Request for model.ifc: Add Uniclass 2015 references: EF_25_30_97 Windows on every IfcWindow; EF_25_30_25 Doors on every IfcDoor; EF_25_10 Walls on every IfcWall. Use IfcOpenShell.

First a look at what the model holds.

```python
import ifcopenshell

model = ifcopenshell.open("model.ifc")
print(model.schema)
print("classifications:", [c.Name for c in model.by_type("IfcClassification")])
for ifc_class in ("IfcDoor", "IfcRoof", "IfcStair", "IfcWall", "IfcWindow"):
    print(ifc_class, len(model.by_type(ifc_class)))
```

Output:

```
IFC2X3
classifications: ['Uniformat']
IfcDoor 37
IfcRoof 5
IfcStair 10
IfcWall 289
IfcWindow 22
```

```python
import ifcopenshell
import ifcopenshell.api.classification

model = ifcopenshell.open("model.ifc")

# IFC2X3 requires Source and Edition and has no link from the project to the system.
system = model.create_entity("IfcClassification", Source="NBS", Edition="2015", Name="Uniclass 2015")

codes = {
    "IfcWindow": ("EF_25_30_97", "Windows"),
    "IfcDoor": ("EF_25_30_25", "Doors"),
    "IfcWall": ("EF_25_10", "Walls"),
}
for ifc_class, (code, name) in codes.items():
    products = model.by_type(ifc_class)
    ifcopenshell.api.classification.add_reference(
        model, products=products, classification=system, identification=code, name=name
    )
    print(code, len(products))

model.write("model_rev.ifc")
```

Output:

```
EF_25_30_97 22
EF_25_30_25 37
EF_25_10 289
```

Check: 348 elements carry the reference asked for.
